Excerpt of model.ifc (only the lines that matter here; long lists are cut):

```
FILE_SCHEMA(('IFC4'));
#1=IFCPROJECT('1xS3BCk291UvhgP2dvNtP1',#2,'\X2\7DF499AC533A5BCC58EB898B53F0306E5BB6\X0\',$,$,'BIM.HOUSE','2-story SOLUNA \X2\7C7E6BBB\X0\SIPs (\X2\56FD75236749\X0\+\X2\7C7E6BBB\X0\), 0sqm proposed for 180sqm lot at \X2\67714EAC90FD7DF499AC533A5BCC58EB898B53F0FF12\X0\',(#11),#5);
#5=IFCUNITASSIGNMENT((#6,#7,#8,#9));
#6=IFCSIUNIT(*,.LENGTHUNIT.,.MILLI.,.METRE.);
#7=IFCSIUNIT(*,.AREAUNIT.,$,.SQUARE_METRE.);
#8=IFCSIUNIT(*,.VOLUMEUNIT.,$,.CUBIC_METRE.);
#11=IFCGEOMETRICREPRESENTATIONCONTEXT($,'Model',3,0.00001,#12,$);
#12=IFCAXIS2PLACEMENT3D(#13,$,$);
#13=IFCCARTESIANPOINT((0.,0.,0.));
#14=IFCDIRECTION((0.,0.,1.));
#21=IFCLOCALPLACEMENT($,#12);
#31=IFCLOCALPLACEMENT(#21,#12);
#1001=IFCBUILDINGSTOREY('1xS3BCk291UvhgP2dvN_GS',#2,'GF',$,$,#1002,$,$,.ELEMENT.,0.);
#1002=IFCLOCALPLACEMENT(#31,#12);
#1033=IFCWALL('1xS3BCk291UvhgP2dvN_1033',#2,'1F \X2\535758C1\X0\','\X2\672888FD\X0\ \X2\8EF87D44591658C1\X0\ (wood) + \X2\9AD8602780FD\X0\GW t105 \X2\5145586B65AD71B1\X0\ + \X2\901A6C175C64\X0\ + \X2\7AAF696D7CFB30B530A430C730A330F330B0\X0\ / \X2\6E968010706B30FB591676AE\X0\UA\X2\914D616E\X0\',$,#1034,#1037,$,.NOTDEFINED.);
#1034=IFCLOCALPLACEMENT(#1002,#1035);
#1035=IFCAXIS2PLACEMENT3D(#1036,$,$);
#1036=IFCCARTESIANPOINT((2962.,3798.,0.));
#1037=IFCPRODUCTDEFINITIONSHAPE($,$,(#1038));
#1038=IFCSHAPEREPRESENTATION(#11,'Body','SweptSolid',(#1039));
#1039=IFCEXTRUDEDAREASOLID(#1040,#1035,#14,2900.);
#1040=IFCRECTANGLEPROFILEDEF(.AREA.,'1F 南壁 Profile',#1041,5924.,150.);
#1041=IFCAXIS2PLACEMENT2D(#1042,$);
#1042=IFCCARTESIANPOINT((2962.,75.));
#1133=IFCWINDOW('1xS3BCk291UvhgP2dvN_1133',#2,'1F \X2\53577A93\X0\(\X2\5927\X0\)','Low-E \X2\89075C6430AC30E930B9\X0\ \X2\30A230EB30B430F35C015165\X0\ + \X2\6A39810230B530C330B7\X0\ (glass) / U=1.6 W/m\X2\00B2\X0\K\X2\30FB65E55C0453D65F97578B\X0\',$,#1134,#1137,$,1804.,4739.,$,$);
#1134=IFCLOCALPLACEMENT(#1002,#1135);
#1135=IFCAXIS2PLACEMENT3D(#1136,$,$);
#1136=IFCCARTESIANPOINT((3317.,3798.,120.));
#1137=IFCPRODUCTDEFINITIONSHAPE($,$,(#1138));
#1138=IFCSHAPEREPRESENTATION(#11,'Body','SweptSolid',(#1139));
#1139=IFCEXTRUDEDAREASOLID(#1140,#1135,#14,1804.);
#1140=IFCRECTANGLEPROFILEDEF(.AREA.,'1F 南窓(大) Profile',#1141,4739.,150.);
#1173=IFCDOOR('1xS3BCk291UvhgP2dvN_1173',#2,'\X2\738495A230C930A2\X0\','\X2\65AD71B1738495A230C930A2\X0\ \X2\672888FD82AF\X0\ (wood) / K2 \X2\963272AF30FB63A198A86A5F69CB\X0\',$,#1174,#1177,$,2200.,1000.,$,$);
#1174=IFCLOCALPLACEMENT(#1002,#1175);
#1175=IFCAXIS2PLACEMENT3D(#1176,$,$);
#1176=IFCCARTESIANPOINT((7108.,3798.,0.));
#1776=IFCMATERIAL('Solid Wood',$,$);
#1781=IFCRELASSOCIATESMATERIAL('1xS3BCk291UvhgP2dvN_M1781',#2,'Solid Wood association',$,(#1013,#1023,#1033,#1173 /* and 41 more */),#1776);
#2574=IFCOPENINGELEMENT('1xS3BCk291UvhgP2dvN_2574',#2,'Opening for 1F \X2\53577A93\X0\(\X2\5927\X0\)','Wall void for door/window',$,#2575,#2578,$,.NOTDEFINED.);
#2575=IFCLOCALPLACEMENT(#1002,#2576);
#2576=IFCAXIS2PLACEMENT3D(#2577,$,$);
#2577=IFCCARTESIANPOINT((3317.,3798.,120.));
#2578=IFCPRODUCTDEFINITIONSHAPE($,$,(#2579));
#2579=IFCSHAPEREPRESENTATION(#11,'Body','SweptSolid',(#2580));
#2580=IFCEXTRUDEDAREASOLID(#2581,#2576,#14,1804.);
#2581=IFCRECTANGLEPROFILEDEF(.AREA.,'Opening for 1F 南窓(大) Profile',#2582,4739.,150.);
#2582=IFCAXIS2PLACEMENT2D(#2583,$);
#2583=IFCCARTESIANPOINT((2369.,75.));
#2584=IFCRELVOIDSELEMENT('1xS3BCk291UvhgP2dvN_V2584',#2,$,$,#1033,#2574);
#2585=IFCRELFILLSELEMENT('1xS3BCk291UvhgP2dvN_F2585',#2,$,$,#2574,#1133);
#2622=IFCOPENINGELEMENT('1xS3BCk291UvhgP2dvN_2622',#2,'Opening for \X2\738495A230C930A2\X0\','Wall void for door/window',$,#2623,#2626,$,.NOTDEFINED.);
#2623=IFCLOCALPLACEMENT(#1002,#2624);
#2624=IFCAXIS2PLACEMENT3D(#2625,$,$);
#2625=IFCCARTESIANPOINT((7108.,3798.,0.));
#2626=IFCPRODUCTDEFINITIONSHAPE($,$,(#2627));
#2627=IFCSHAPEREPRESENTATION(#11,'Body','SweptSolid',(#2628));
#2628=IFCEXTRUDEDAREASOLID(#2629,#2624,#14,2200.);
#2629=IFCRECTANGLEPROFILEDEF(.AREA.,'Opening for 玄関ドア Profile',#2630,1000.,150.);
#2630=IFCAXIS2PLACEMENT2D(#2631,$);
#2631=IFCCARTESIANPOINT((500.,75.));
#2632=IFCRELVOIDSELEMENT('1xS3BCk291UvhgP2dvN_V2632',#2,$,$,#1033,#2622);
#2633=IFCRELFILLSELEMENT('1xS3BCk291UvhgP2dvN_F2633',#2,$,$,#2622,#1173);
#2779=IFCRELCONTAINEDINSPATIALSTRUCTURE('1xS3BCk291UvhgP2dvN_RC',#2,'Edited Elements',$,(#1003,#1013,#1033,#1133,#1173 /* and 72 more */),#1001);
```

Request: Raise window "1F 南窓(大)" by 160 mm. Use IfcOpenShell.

```python
import numpy as np
import ifcopenshell
import ifcopenshell.api.geometry
import ifcopenshell.util.placement
import ifcopenshell.util.unit

model = ifcopenshell.open("model.ifc")
unit_scale = ifcopenshell.util.unit.calculate_unit_scale(model)

window = model.by_guid("1xS3BCk291UvhgP2dvN_1133")
opening = window.FillsVoids[0].RelatingOpeningElement
dz = 160.0

shift = np.array([0.0, 0.0, dz])
# The window is not placed relative to its opening, so move both.
for product in (opening, window):
    matrix = ifcopenshell.util.placement.get_local_placement(product.ObjectPlacement)
    matrix[:3, 3] += shift
    ifcopenshell.api.geometry.edit_object_placement(model, product=product, matrix=matrix, is_si=False)

print(f"moved by {dz * unit_scale:+.3f} m")

model.write("model_updated.ifc")
```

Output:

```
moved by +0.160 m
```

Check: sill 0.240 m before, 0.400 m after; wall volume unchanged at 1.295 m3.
